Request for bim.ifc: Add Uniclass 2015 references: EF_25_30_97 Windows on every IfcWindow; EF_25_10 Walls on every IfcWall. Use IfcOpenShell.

First a look at what the model holds.

```python
import ifcopenshell

model = ifcopenshell.open("bim.ifc")
print(model.schema)
print("classifications:", [c.Name for c in model.by_type("IfcClassification")])
for ifc_class in ("IfcDoor", "IfcRoof", "IfcStair", "IfcWall", "IfcWindow"):
    print(ifc_class, len(model.by_type(ifc_class)))
```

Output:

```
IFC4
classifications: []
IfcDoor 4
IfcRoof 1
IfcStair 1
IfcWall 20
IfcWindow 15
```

```python
import ifcopenshell
import ifcopenshell.api.classification

model = ifcopenshell.open("bim.ifc")

system = ifcopenshell.api.classification.add_classification(model, classification="Uniclass 2015")

codes = {
    "IfcWindow": ("EF_25_30_97", "Windows"),
    "IfcWall": ("EF_25_10", "Walls"),
}
for ifc_class, (code, name) in codes.items():
    products = model.by_type(ifc_class)
    ifcopenshell.api.classification.add_reference(
        model, products=products, classification=system, identification=code, name=name
    )
    print(code, len(products))

model.write("bim-out.ifc")
```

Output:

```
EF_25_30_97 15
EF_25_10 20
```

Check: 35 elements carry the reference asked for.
